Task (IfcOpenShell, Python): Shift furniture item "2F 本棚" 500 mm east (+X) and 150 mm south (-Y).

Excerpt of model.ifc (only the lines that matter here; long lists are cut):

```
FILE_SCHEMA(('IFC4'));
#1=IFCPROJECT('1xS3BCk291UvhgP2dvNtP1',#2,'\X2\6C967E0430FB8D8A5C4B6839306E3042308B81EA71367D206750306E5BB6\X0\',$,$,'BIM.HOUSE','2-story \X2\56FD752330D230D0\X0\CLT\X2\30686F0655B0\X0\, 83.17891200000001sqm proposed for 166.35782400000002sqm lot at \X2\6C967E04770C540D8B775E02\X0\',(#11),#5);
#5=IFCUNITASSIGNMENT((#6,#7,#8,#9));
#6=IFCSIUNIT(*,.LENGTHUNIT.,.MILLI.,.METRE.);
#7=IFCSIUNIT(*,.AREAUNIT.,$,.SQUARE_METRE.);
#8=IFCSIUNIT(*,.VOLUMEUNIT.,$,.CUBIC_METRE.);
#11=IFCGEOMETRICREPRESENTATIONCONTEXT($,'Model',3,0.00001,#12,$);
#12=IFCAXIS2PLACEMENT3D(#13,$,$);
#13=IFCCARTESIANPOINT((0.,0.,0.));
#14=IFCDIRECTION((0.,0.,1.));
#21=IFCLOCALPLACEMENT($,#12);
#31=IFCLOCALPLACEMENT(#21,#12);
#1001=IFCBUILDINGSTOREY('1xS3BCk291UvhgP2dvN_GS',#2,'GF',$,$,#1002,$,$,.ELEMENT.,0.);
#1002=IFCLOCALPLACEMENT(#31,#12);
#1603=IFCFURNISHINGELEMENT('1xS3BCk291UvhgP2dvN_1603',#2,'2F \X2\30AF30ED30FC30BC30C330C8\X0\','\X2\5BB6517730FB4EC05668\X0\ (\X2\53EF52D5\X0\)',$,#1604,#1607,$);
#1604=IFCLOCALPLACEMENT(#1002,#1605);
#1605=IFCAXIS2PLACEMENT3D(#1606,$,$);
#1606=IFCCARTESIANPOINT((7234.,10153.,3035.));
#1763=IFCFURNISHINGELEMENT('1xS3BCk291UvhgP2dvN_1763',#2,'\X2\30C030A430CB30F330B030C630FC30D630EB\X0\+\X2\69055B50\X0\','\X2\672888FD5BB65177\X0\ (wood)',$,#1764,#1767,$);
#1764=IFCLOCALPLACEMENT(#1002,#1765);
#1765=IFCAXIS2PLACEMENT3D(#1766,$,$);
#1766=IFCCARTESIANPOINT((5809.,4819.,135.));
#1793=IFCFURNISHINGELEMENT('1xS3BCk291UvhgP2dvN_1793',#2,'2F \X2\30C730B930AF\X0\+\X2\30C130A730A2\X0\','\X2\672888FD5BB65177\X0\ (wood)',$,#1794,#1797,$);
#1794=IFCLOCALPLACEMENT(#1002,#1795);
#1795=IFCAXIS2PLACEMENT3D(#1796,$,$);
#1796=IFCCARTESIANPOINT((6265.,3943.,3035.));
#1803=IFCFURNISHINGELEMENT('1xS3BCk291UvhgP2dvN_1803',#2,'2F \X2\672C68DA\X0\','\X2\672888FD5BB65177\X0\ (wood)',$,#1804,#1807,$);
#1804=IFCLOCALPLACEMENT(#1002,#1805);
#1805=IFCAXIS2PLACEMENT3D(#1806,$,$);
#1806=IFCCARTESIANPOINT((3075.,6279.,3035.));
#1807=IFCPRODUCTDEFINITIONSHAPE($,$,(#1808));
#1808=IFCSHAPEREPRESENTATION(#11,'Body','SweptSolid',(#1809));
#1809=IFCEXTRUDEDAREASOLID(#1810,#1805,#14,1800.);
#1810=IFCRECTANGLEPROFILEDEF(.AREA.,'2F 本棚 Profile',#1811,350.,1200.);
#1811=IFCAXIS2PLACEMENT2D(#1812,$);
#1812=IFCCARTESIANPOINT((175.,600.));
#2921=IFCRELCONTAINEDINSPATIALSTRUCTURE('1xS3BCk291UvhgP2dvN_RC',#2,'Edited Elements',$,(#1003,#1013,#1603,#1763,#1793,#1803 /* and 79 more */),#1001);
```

```python
import ifcopenshell
import ifcopenshell.api.geometry
import ifcopenshell.util.placement

model = ifcopenshell.open("model.ifc")

item = model.by_id(1803)
matrix = ifcopenshell.util.placement.get_local_placement(item.ObjectPlacement)
matrix[0, 3] += 500.0
matrix[1, 3] -= 150.0
ifcopenshell.api.geometry.edit_object_placement(model, product=item, matrix=matrix, is_si=False)

print(ifcopenshell.util.placement.get_local_placement(item.ObjectPlacement).round(3) + 0.0)

model.write("model_rev.ifc")
```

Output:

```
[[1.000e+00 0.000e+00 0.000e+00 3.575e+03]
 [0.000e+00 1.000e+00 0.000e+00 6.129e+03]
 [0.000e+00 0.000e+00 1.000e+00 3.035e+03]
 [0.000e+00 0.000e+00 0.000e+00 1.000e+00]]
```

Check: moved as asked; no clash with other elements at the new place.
